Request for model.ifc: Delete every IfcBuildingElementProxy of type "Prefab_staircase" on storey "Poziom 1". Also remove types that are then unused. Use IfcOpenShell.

First a look at what the model holds.

```python
import ifcopenshell
import ifcopenshell.util.element

model = ifcopenshell.open("model.ifc")
print(model.schema)
storey = next(s for s in model.by_type("IfcBuildingStorey") if s.Name == "Poziom 1")
proxies = [e for e in ifcopenshell.util.element.get_decomposition(storey) if e.is_a("IfcBuildingElementProxy")]
seen = {}
for e in proxies:
    element_type = ifcopenshell.util.element.get_type(e)
    name = element_type.Name if element_type not in (None, e) else None
    seen[name] = seen.get(name, 0) + 1
for name, count in sorted(seen.items(), key=str):
    print(count, "x", name)
```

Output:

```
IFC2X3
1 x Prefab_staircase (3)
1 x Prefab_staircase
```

```python
import ifcopenshell
import ifcopenshell.api.root
import ifcopenshell.util.element

model = ifcopenshell.open("model.ifc")

storey = next(s for s in model.by_type("IfcBuildingStorey") if s.Name == "Poziom 1")
proxies = [e for e in ifcopenshell.util.element.get_decomposition(storey) if e.is_a("IfcBuildingElementProxy")]
targets = [e for e in proxies if (t := ifcopenshell.util.element.get_type(e)) not in (None, e) and t.Name == "Prefab_staircase"]
types = {ifcopenshell.util.element.get_type(e) for e in targets} - {None, *targets}

for e in targets:
    ifcopenshell.api.root.remove_product(model, product=e)
print(len(targets), "removed")

unused = [t for t in types if not ifcopenshell.util.element.get_types(t)]
for t in unused:
    ifcopenshell.api.root.remove_product(model, product=t)
print(len(unused), "unused types removed")

model.write("model-out.ifc")
```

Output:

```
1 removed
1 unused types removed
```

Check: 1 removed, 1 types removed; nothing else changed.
